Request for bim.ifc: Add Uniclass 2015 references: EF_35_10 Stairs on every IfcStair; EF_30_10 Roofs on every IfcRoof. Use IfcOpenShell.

First a look at what the model holds.

```python
import ifcopenshell

model = ifcopenshell.open("bim.ifc")
print(model.schema)
print("classifications:", [c.Name for c in model.by_type("IfcClassification")])
for ifc_class in ("IfcDoor", "IfcRoof", "IfcStair", "IfcWall", "IfcWindow"):
    print(ifc_class, len(model.by_type(ifc_class)))
```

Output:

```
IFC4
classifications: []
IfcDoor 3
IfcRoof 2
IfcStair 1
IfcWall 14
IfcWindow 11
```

```python
import ifcopenshell
import ifcopenshell.api.classification

model = ifcopenshell.open("bim.ifc")

system = ifcopenshell.api.classification.add_classification(model, classification="Uniclass 2015")

codes = {
    "IfcStair": ("EF_35_10", "Stairs"),
    "IfcRoof": ("EF_30_10", "Roofs"),
}
for ifc_class, (code, name) in codes.items():
    products = model.by_type(ifc_class)
    ifcopenshell.api.classification.add_reference(
        model, products=products, classification=system, identification=code, name=name
    )
    print(code, len(products))

model.write("bim_rev.ifc")
```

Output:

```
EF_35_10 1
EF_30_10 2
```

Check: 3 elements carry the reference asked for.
